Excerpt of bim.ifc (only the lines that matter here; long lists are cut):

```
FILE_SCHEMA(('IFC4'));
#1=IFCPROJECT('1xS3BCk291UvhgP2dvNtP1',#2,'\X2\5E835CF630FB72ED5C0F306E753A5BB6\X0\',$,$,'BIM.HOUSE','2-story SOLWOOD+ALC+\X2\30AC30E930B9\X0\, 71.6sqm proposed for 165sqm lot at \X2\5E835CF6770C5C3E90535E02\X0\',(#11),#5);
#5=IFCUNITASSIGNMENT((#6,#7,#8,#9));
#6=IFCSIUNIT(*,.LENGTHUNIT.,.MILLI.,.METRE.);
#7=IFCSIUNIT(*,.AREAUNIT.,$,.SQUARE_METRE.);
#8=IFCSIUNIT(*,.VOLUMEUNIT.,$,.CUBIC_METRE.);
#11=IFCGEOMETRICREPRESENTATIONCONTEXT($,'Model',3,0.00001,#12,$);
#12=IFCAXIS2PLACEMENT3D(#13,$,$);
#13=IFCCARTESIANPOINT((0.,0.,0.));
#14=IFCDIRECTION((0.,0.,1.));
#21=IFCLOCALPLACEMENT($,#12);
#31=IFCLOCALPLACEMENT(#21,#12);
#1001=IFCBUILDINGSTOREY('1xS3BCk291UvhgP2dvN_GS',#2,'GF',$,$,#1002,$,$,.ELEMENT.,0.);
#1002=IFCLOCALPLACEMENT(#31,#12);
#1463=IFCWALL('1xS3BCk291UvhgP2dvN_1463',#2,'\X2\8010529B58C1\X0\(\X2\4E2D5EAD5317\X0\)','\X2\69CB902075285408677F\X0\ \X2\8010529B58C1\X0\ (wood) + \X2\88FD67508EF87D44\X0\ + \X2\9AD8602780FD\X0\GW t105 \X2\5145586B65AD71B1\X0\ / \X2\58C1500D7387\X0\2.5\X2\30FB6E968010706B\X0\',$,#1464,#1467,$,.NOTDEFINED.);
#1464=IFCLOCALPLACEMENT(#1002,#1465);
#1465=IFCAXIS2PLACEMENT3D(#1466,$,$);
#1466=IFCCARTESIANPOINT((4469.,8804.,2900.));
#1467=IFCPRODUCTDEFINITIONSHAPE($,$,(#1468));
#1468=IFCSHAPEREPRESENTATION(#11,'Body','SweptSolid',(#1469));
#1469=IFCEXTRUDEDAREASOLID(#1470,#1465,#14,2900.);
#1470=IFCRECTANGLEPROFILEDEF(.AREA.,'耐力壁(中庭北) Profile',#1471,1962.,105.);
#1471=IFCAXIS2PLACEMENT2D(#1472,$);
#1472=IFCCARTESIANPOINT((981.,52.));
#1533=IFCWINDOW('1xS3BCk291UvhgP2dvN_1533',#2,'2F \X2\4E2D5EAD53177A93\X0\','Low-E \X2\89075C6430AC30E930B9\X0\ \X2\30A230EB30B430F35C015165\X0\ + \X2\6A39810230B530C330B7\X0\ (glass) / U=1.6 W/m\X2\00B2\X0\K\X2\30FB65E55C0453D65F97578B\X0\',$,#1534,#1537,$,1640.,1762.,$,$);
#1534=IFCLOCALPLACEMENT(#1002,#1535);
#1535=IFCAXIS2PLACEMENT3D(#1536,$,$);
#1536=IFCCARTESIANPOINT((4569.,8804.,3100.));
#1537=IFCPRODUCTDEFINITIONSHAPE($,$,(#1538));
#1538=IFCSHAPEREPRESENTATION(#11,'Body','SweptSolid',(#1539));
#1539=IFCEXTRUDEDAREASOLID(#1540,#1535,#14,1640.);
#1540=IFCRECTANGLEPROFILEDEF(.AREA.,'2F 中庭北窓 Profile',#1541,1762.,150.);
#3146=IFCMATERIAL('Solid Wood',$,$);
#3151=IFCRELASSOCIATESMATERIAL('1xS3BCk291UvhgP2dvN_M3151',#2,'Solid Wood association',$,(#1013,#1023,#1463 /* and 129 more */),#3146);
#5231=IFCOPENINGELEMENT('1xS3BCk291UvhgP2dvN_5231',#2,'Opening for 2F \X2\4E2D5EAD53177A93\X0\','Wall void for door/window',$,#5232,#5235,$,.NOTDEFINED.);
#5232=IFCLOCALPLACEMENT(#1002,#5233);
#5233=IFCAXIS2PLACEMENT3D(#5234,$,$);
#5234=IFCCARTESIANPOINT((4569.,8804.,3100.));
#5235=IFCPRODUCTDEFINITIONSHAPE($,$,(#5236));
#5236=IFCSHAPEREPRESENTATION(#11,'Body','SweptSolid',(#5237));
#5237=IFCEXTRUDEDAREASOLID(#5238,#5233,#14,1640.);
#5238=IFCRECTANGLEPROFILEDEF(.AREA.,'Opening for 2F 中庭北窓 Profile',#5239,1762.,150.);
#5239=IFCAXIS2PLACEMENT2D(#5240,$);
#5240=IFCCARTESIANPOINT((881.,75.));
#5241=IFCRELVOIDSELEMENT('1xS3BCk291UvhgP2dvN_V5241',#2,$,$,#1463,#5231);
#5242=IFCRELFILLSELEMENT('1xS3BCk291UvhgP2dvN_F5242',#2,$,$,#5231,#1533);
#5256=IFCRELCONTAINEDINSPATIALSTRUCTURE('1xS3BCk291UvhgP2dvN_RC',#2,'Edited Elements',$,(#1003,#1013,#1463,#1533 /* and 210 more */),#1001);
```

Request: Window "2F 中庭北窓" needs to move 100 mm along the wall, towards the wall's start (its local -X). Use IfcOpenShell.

```python
import ifcopenshell
import ifcopenshell.api.geometry
import ifcopenshell.util.placement
import ifcopenshell.util.unit

model = ifcopenshell.open("bim.ifc")
unit_scale = ifcopenshell.util.unit.calculate_unit_scale(model)

window = model.by_guid("1xS3BCk291UvhgP2dvN_1533")
opening = window.FillsVoids[0].RelatingOpeningElement
wall = opening.VoidsElements[0].RelatingBuildingElement

wall_matrix = ifcopenshell.util.placement.get_local_placement(wall.ObjectPlacement)
shift = wall_matrix[:3, 0] * -0.1 / unit_scale
before = ifcopenshell.util.placement.get_local_placement(window.ObjectPlacement)[:3, 3].copy()

# The window is not placed relative to its opening, so move both.
for product in (opening, window):
    matrix = ifcopenshell.util.placement.get_local_placement(product.ObjectPlacement)
    matrix[:3, 3] += shift
    ifcopenshell.api.geometry.edit_object_placement(model, product=product, matrix=matrix, is_si=False)

after = ifcopenshell.util.placement.get_local_placement(window.ObjectPlacement)[:3, 3]
print("window moved by", (after - before).round(3) + 0.0)

model.write("bim_edited.ifc")
```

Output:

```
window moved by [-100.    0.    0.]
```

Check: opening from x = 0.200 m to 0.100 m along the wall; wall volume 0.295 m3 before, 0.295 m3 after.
